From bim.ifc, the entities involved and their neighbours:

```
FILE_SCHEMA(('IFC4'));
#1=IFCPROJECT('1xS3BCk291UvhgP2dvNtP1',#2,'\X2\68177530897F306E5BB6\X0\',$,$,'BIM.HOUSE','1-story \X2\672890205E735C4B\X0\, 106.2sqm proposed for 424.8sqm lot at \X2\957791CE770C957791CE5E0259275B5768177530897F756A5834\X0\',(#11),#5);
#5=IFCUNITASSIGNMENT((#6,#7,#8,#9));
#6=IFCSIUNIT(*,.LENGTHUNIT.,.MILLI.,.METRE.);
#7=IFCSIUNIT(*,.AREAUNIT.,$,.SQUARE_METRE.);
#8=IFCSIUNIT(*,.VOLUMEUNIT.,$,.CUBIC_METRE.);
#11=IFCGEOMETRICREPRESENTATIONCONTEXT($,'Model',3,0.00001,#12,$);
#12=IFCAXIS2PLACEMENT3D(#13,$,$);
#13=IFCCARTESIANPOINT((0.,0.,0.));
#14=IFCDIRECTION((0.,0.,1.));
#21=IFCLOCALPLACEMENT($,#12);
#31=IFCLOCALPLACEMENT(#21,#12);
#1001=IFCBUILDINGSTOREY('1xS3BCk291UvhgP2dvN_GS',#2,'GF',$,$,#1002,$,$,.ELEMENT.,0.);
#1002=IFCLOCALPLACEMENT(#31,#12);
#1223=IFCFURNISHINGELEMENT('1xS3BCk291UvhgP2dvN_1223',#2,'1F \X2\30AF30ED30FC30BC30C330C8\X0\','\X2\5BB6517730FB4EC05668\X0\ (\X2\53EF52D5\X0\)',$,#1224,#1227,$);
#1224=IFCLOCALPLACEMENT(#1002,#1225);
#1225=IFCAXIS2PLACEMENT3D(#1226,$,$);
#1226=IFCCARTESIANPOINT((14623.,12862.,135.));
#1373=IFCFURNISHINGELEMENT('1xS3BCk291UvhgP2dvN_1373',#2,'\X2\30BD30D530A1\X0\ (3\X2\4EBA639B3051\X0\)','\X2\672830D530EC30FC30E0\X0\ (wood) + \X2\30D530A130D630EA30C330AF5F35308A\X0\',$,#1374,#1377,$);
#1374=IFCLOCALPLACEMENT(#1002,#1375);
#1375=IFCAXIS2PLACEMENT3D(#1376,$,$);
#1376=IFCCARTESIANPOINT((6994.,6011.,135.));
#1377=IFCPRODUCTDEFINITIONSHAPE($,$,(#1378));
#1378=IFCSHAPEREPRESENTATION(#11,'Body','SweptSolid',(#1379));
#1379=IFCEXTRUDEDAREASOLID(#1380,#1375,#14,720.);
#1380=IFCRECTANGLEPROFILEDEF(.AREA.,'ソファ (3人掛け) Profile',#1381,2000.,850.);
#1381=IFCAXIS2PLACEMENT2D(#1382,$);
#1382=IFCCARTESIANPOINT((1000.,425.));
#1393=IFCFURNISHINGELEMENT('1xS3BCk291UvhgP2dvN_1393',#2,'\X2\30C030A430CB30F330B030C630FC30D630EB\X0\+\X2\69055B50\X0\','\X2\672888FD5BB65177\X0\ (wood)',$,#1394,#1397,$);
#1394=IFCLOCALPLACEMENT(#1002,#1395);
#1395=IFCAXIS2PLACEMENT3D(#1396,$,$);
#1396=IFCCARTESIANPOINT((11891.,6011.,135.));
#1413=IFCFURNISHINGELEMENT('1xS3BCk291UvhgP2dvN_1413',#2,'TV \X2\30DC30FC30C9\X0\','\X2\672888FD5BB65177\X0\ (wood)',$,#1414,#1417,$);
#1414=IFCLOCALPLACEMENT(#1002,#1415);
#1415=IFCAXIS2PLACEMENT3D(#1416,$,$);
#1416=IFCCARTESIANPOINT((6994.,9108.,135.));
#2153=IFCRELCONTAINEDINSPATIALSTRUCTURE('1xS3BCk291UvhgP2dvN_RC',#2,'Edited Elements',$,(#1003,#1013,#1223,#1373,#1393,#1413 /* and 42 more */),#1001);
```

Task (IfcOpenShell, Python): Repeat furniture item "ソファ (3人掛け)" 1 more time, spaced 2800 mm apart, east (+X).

```python
import numpy as np
import ifcopenshell
import ifcopenshell.api.geometry
import ifcopenshell.api.root
import ifcopenshell.util.element
import ifcopenshell.util.placement

model = ifcopenshell.open("bim.ifc")


def reuse_history(source, copy):
    """copy_class also copies each property set's owner history, people and application; keep the originals."""
    for rel in copy.IsDefinedBy:
        if rel.is_a("IfcRelDefinesByProperties") and (history := rel.RelatingPropertyDefinition.OwnerHistory):
            rel.RelatingPropertyDefinition.OwnerHistory = source.OwnerHistory
            ifcopenshell.util.element.remove_deep2(model, history)


source = model.by_guid("1xS3BCk291UvhgP2dvN_1373")
base = ifcopenshell.util.placement.get_local_placement(source.ObjectPlacement)
step = np.array([1.0, 0.0, 0.0]) * 2800.0

for i in range(1, 2):
    copy = ifcopenshell.api.root.copy_class(model, product=source)
    copy.Representation = ifcopenshell.util.element.copy_deep(
        model, source.Representation, exclude=["IfcGeometricRepresentationContext", "IfcRepresentationMap"]
    )
    reuse_history(source, copy)
    matrix = base.copy()
    matrix[:3, 3] += i * step
    print("added at", matrix[:3, 3].round(3) + 0.0)
    ifcopenshell.api.geometry.edit_object_placement(model, product=copy, matrix=matrix, is_si=False)

model.write("bim_updated.ifc")
```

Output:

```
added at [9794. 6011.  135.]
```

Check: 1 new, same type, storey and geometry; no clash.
